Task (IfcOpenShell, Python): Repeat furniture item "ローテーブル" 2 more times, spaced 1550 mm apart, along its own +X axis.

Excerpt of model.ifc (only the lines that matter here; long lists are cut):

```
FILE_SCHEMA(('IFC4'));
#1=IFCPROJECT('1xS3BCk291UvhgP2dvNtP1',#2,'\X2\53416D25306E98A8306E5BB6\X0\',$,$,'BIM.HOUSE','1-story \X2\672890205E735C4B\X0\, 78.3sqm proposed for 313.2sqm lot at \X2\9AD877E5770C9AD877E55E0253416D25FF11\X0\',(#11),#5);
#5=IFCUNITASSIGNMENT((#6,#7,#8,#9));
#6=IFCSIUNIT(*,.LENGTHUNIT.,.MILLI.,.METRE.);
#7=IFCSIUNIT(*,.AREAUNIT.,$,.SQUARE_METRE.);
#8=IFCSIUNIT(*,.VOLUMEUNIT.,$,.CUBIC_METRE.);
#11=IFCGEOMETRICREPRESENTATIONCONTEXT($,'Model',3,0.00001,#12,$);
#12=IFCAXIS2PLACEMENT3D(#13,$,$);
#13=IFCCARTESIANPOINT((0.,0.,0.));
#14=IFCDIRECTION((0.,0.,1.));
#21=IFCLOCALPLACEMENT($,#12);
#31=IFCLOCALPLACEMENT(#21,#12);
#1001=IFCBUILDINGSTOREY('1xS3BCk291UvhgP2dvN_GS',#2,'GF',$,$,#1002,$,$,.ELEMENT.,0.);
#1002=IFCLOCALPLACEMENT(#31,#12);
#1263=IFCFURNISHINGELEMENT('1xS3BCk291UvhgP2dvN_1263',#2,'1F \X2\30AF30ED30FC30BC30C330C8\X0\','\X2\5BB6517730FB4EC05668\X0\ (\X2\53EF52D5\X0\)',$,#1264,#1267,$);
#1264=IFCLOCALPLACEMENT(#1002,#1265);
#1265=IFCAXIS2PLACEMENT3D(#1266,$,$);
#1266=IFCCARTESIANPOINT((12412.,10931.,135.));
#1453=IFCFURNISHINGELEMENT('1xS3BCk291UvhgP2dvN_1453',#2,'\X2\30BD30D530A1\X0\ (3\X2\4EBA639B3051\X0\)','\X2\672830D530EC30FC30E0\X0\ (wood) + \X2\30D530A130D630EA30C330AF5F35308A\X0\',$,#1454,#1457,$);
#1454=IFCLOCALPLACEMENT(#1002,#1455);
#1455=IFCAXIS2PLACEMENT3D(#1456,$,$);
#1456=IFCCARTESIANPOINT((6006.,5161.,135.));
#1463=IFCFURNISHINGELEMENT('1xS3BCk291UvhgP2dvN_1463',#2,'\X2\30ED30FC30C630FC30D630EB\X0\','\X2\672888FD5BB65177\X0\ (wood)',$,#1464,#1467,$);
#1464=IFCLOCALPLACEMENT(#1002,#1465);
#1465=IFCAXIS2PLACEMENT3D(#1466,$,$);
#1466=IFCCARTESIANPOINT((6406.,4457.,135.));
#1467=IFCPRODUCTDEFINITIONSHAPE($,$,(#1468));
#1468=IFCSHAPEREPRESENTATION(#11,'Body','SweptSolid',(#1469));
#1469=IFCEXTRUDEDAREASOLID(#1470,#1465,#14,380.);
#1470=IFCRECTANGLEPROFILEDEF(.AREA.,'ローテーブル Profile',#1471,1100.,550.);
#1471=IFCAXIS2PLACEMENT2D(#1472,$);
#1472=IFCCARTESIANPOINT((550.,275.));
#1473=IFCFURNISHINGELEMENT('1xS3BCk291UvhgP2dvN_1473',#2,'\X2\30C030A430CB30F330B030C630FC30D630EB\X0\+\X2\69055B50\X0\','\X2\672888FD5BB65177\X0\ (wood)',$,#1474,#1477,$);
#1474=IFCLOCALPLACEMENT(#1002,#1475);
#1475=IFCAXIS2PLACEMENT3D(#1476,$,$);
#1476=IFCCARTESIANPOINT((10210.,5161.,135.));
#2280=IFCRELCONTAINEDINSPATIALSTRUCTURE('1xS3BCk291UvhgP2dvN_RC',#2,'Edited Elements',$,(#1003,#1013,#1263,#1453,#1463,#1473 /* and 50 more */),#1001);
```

```python
import ifcopenshell
import ifcopenshell.api.geometry
import ifcopenshell.api.root
import ifcopenshell.util.element
import ifcopenshell.util.placement
import ifcopenshell.util.unit

model = ifcopenshell.open("model.ifc")
unit_scale = ifcopenshell.util.unit.calculate_unit_scale(model)


def reuse_history(source, copy):
    """copy_class also copies each property set's owner history, people and application; keep the originals."""
    for rel in copy.IsDefinedBy:
        if rel.is_a("IfcRelDefinesByProperties") and (history := rel.RelatingPropertyDefinition.OwnerHistory):
            rel.RelatingPropertyDefinition.OwnerHistory = source.OwnerHistory
            ifcopenshell.util.element.remove_deep2(model, history)


source = model.by_guid("1xS3BCk291UvhgP2dvN_1463")
base = ifcopenshell.util.placement.get_local_placement(source.ObjectPlacement)
step = base[:3, 0] * 1.55 / unit_scale

for i in range(1, 3):
    copy = ifcopenshell.api.root.copy_class(model, product=source)
    copy.Representation = ifcopenshell.util.element.copy_deep(
        model, source.Representation, exclude=["IfcGeometricRepresentationContext", "IfcRepresentationMap"]
    )
    reuse_history(source, copy)
    matrix = base.copy()
    matrix[:3, 3] += i * step
    print("added at", matrix[:3, 3].round(3) + 0.0)
    ifcopenshell.api.geometry.edit_object_placement(model, product=copy, matrix=matrix, is_si=False)

model.write("model_edited.ifc")
```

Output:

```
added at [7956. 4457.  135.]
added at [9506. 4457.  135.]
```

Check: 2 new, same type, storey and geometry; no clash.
